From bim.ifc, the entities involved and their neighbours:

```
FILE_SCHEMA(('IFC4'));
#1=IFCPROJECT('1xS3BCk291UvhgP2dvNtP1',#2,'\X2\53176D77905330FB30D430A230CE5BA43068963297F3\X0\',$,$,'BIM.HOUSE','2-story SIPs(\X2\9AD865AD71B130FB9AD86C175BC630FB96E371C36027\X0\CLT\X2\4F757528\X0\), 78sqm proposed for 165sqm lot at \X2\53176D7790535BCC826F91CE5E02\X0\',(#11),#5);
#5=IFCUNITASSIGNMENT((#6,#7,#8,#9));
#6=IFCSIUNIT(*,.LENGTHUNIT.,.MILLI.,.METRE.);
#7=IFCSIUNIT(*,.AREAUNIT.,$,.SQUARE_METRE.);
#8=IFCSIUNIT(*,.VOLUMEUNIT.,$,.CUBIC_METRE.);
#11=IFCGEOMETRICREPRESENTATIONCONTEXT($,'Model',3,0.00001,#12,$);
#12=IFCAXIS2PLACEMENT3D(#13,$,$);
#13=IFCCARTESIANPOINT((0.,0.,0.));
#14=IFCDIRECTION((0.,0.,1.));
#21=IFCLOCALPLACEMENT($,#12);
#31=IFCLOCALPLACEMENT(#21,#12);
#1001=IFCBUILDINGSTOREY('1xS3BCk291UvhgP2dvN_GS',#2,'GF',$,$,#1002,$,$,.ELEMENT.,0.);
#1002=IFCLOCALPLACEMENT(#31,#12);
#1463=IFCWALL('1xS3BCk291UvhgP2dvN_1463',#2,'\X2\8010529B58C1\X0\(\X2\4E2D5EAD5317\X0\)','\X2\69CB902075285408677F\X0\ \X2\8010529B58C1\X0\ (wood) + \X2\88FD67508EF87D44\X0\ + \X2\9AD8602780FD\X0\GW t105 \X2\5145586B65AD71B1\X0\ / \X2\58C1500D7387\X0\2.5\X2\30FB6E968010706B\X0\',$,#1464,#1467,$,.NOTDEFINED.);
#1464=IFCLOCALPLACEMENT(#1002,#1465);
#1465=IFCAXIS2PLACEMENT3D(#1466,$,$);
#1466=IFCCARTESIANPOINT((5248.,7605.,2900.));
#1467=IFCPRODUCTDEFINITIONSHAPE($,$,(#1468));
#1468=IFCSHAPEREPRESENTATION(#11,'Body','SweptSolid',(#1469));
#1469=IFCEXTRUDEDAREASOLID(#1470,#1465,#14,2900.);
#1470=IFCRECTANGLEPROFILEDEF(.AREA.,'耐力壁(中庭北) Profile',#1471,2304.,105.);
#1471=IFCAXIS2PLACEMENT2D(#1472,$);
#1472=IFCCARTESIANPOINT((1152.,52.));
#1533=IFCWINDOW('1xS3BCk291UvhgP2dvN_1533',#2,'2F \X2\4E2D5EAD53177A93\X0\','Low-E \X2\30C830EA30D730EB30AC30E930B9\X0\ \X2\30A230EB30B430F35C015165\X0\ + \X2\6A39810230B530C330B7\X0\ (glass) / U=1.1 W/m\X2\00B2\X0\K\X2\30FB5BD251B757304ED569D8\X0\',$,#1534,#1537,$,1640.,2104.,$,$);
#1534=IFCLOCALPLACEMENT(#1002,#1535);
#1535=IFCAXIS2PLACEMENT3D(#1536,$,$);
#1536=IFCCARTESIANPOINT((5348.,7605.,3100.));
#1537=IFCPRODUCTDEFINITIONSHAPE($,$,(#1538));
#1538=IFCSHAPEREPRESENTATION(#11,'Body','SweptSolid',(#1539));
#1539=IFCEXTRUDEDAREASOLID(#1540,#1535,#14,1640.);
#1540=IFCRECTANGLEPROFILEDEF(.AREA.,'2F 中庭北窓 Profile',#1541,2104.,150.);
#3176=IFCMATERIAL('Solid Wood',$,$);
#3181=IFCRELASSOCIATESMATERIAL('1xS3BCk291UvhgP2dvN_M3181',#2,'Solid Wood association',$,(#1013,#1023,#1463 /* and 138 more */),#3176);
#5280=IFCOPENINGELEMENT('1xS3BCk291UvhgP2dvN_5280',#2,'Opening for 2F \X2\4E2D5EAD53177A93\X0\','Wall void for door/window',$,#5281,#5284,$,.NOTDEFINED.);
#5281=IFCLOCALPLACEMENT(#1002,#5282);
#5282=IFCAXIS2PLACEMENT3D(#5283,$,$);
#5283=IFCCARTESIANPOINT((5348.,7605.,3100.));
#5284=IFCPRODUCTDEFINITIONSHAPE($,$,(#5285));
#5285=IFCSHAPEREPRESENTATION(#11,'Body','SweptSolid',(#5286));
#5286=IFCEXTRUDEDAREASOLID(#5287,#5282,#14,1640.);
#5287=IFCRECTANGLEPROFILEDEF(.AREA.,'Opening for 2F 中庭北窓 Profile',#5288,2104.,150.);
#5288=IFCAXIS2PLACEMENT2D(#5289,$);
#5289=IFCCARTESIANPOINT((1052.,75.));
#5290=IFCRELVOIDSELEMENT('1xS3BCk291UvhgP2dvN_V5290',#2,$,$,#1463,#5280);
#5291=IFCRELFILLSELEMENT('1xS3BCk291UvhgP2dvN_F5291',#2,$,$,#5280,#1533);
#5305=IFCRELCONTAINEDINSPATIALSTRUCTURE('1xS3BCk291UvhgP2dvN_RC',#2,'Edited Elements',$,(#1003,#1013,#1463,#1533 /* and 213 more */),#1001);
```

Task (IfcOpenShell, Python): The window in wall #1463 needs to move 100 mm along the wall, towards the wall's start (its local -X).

```python
import ifcopenshell
import ifcopenshell.api.geometry
import ifcopenshell.util.placement
import ifcopenshell.util.unit

model = ifcopenshell.open("bim.ifc")
unit_scale = ifcopenshell.util.unit.calculate_unit_scale(model)

window = model.by_guid("1xS3BCk291UvhgP2dvN_1533")
opening = window.FillsVoids[0].RelatingOpeningElement
wall = opening.VoidsElements[0].RelatingBuildingElement

wall_matrix = ifcopenshell.util.placement.get_local_placement(wall.ObjectPlacement)
shift = wall_matrix[:3, 0] * -0.1 / unit_scale
before = ifcopenshell.util.placement.get_local_placement(window.ObjectPlacement)[:3, 3].copy()

# The window is not placed relative to its opening, so move both.
for product in (opening, window):
    matrix = ifcopenshell.util.placement.get_local_placement(product.ObjectPlacement)
    matrix[:3, 3] += shift
    ifcopenshell.api.geometry.edit_object_placement(model, product=product, matrix=matrix, is_si=False)

after = ifcopenshell.util.placement.get_local_placement(window.ObjectPlacement)[:3, 3]
print("window moved by", (after - before).round(3) + 0.0)

model.write("bim_rev.ifc")
```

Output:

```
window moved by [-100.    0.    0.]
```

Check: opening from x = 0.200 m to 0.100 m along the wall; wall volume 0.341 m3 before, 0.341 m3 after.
